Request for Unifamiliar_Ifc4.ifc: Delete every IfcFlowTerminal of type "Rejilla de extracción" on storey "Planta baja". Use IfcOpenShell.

First a look at what the model holds.

```python
import ifcopenshell
import ifcopenshell.util.element

model = ifcopenshell.open("Unifamiliar_Ifc4.ifc")
print(model.schema)
storey = next(s for s in model.by_type("IfcBuildingStorey") if s.Name == "Planta baja")
terminals = [e for e in ifcopenshell.util.element.get_decomposition(storey) if e.is_a("IfcFlowTerminal")]
seen = {}
for e in terminals:
    element_type = ifcopenshell.util.element.get_type(e)
    name = element_type.Name if element_type not in (None, e) else None
    seen[name] = seen.get(name, 0) + 1
for name, count in sorted(seen.items(), key=str):
    print(count, "x", name)
```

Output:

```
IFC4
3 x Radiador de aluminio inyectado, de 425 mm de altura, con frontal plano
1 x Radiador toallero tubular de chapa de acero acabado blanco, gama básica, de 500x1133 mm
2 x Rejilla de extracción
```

```python
import ifcopenshell
import ifcopenshell.api.root
import ifcopenshell.util.element

model = ifcopenshell.open("Unifamiliar_Ifc4.ifc")

storey = next(s for s in model.by_type("IfcBuildingStorey") if s.Name == "Planta baja")
terminals = [e for e in ifcopenshell.util.element.get_decomposition(storey) if e.is_a("IfcFlowTerminal")]
targets = [e for e in terminals if (t := ifcopenshell.util.element.get_type(e)) not in (None, e) and t.Name == "Rejilla de extracción"]

for e in targets:
    ifcopenshell.api.root.remove_product(model, product=e)
print(len(targets), "removed")

model.write("Unifamiliar_Ifc4_rev.ifc")
```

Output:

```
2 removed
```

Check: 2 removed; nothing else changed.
